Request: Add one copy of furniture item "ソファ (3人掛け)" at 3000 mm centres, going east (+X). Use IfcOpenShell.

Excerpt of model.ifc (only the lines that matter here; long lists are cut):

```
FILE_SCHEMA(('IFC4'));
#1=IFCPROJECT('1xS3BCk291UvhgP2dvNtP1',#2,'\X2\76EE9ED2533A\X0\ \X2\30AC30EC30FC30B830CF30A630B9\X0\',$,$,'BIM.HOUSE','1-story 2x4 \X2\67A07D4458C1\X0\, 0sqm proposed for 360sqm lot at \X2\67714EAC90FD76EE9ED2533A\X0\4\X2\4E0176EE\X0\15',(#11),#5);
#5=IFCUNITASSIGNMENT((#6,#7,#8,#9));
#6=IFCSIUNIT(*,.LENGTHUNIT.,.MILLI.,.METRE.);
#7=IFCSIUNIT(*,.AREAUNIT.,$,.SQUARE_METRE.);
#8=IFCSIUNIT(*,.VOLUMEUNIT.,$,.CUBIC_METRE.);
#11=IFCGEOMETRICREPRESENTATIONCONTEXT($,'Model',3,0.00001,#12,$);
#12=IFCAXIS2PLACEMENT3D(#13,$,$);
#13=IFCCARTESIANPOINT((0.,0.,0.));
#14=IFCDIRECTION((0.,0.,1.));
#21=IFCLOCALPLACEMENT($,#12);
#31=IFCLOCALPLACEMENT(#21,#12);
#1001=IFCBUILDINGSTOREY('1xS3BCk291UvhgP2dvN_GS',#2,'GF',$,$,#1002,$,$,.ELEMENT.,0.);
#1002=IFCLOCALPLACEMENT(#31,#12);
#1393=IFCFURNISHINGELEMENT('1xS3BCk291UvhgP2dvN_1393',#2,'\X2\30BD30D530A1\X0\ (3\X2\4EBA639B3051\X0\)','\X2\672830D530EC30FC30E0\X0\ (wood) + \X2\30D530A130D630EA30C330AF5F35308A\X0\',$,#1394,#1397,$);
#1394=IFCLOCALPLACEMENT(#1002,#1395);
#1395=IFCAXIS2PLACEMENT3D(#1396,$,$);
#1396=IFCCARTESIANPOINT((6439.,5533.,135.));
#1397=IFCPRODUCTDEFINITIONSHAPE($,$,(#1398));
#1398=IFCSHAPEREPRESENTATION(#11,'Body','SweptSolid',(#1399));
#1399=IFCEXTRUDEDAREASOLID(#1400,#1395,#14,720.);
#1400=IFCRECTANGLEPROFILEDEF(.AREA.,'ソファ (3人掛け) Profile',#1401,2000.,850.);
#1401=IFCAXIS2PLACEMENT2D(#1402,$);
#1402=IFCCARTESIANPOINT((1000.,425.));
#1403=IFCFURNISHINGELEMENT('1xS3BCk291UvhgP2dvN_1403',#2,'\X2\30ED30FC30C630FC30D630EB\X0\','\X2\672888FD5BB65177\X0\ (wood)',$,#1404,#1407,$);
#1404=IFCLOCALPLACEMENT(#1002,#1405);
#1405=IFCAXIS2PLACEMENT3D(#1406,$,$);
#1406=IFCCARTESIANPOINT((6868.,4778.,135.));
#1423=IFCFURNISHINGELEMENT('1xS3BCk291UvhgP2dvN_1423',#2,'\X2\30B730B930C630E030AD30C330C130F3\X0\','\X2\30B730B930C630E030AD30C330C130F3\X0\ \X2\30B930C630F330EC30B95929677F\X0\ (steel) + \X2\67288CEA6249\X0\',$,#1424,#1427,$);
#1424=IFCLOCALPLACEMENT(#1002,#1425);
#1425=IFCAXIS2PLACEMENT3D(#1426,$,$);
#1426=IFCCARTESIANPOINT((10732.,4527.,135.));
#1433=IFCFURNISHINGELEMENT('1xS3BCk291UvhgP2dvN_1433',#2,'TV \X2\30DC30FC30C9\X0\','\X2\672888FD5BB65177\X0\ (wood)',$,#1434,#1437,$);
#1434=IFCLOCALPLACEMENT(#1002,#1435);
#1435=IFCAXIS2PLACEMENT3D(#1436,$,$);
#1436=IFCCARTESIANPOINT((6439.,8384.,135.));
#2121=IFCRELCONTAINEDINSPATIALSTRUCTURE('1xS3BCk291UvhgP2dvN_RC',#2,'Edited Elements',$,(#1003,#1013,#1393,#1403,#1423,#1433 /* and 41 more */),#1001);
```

```python
import numpy as np
import ifcopenshell
import ifcopenshell.api.geometry
import ifcopenshell.api.root
import ifcopenshell.util.element
import ifcopenshell.util.placement
import ifcopenshell.util.unit

model = ifcopenshell.open("model.ifc")
unit_scale = ifcopenshell.util.unit.calculate_unit_scale(model)


def reuse_history(source, copy):
    """copy_class also copies each property set's owner history, people and application; keep the originals."""
    for rel in copy.IsDefinedBy:
        if rel.is_a("IfcRelDefinesByProperties") and (history := rel.RelatingPropertyDefinition.OwnerHistory):
            rel.RelatingPropertyDefinition.OwnerHistory = source.OwnerHistory
            ifcopenshell.util.element.remove_deep2(model, history)


source = model.by_id(1393)
base = ifcopenshell.util.placement.get_local_placement(source.ObjectPlacement)
step = np.array([1.0, 0.0, 0.0]) * 3 / unit_scale

for i in range(1, 2):
    copy = ifcopenshell.api.root.copy_class(model, product=source)
    copy.Representation = ifcopenshell.util.element.copy_deep(
        model, source.Representation, exclude=["IfcGeometricRepresentationContext", "IfcRepresentationMap"]
    )
    reuse_history(source, copy)
    matrix = base.copy()
    matrix[:3, 3] += i * step
    print("added at", matrix[:3, 3].round(3) + 0.0)
    ifcopenshell.api.geometry.edit_object_placement(model, product=copy, matrix=matrix, is_si=False)

model.write("model_v2.ifc")
```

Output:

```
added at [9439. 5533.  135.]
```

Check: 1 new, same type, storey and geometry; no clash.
